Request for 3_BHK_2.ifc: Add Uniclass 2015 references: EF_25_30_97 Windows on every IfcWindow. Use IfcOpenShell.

First a look at what the model holds.

```python
import ifcopenshell

model = ifcopenshell.open("3_BHK_2.ifc")
print(model.schema)
print("classifications:", [c.Name for c in model.by_type("IfcClassification")])
for ifc_class in ("IfcDoor", "IfcRoof", "IfcStair", "IfcWall", "IfcWindow"):
    print(ifc_class, len(model.by_type(ifc_class)))
```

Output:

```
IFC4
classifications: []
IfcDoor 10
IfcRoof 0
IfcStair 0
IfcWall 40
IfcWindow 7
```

```python
import ifcopenshell
import ifcopenshell.api.classification

model = ifcopenshell.open("3_BHK_2.ifc")

system = ifcopenshell.api.classification.add_classification(model, classification="Uniclass 2015")

codes = {
    "IfcWindow": ("EF_25_30_97", "Windows"),
}
for ifc_class, (code, name) in codes.items():
    products = model.by_type(ifc_class)
    ifcopenshell.api.classification.add_reference(
        model, products=products, classification=system, identification=code, name=name
    )
    print(code, len(products))

model.write("3_BHK_2_rev.ifc")
```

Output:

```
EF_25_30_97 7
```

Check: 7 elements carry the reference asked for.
